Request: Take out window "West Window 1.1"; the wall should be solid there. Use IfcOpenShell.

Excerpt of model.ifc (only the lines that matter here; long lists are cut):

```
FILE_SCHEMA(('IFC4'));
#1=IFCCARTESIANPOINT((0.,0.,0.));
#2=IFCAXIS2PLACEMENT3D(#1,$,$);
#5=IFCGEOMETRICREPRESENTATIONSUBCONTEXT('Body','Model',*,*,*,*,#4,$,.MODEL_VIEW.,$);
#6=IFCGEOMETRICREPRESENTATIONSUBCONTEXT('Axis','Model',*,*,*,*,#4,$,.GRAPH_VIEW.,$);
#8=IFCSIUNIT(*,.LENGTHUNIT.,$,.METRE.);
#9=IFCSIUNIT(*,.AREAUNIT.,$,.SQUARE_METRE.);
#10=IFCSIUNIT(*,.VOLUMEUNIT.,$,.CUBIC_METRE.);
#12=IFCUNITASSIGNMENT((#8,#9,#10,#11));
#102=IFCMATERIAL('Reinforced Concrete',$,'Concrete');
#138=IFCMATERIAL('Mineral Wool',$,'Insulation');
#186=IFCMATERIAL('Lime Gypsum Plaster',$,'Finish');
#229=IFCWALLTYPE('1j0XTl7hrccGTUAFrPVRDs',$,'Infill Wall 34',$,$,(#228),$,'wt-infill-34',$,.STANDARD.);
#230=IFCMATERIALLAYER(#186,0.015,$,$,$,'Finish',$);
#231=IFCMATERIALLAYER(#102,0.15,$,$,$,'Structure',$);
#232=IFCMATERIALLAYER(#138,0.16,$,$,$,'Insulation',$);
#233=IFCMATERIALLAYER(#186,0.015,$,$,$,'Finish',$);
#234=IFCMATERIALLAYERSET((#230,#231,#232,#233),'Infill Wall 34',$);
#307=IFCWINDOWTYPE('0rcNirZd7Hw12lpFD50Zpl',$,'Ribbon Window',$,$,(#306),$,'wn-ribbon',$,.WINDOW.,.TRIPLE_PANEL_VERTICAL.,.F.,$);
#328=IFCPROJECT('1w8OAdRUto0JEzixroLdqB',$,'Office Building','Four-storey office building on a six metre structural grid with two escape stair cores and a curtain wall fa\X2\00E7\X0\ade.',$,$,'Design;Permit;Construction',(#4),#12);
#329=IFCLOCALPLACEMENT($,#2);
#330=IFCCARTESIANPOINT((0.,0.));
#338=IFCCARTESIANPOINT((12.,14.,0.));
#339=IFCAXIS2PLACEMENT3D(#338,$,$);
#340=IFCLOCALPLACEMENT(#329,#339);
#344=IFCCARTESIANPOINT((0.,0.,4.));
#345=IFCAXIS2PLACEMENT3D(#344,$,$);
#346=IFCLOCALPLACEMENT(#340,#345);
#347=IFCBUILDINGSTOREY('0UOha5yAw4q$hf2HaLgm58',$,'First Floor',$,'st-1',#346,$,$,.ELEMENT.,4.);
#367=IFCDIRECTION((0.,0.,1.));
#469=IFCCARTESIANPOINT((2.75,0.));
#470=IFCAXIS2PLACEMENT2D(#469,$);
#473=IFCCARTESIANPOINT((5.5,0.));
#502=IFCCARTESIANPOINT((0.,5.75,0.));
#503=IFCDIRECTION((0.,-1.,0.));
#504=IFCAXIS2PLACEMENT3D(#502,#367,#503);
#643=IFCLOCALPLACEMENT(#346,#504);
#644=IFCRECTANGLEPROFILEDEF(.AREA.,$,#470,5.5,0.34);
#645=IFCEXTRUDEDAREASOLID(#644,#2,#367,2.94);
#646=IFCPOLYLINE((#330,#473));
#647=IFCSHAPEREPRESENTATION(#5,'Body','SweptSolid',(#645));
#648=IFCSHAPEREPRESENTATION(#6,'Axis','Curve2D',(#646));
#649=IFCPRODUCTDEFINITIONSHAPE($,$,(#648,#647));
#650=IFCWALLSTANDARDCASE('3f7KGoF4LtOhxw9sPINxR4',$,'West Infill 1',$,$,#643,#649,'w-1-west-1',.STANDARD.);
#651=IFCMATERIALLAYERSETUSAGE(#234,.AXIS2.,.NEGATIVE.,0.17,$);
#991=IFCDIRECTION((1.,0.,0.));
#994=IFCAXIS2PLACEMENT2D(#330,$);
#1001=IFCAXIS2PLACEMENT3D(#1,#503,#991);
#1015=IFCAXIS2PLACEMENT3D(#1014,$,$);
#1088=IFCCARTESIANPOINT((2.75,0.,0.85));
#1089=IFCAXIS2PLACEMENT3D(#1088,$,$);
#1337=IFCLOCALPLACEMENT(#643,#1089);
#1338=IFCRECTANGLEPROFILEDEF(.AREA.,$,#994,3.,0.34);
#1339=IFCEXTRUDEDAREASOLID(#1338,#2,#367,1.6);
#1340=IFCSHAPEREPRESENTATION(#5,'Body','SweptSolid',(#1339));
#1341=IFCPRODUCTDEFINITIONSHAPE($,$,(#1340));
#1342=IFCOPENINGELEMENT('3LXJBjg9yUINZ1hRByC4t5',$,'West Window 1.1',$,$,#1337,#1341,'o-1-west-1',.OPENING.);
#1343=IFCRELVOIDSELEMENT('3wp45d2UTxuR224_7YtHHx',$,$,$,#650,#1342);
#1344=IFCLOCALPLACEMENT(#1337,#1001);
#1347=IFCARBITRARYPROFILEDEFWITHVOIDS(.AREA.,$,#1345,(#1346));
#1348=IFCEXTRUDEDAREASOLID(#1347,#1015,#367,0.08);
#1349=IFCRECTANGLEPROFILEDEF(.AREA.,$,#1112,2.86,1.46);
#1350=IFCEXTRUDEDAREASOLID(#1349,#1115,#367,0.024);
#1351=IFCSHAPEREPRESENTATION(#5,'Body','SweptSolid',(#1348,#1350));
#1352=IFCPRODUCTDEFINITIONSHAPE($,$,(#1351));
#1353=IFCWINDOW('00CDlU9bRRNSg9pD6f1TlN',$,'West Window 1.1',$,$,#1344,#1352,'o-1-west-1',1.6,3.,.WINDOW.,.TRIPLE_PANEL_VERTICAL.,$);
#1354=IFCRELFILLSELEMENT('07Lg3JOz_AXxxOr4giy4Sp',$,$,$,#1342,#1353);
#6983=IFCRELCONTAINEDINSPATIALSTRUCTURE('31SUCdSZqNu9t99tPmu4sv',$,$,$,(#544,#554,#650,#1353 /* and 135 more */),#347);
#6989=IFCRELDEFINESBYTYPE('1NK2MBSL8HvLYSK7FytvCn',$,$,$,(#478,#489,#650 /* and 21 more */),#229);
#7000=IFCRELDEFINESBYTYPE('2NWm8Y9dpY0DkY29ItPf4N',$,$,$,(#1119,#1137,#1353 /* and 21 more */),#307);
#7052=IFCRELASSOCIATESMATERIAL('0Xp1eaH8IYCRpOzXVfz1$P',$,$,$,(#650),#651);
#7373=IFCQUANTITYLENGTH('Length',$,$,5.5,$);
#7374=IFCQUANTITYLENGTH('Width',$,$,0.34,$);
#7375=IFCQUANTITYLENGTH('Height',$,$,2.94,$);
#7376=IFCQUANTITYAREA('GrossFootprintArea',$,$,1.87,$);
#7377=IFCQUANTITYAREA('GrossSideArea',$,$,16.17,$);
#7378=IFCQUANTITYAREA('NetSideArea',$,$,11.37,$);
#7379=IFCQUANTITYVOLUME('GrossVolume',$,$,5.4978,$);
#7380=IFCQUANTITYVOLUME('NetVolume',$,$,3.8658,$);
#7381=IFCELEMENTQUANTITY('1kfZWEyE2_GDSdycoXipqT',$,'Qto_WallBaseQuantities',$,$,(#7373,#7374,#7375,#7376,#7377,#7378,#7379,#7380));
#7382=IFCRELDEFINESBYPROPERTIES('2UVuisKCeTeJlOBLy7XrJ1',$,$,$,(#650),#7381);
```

```python
import ifcopenshell
import ifcopenshell.api.feature
import ifcopenshell.api.pset
import ifcopenshell.api.root
import ifcopenshell.geom
import ifcopenshell.util.element
import ifcopenshell.util.shape
import ifcopenshell.util.unit

model = ifcopenshell.open("model.ifc")
area_scale = ifcopenshell.util.unit.calculate_unit_scale(model, "AREAUNIT")
volume_scale = ifcopenshell.util.unit.calculate_unit_scale(model, "VOLUMEUNIT")
settings = ifcopenshell.geom.settings()


def volume(element):
    """Net volume in cubic metres, openings subtracted."""
    shape = ifcopenshell.geom.create_shape(settings, element)
    return ifcopenshell.util.shape.get_volume(shape.geometry)


window = model.by_id(1353)
opening = window.FillsVoids[0].RelatingOpeningElement
wall = opening.VoidsElements[0].RelatingBuildingElement
before = volume(wall)

ifcopenshell.api.root.remove_product(model, product=window)
ifcopenshell.api.feature.remove_feature(model, feature=opening)

after = volume(wall)
thickness = 0.34  # wall thickness in metres

# Update the wall's stored quantities.
qto = model.by_id(ifcopenshell.util.element.get_pset(wall, "Qto_WallBaseQuantities", should_inherit=False)["id"])
ifcopenshell.api.pset.edit_qto(model, qto=qto, properties={
    "NetSideArea": after / thickness / area_scale,
    "NetVolume": after / volume_scale,
})

print(f"wall volume {before:.3f} -> {after:.3f} m3")

model.write("model-out.ifc")
```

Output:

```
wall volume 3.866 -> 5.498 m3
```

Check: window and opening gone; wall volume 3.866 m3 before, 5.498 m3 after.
